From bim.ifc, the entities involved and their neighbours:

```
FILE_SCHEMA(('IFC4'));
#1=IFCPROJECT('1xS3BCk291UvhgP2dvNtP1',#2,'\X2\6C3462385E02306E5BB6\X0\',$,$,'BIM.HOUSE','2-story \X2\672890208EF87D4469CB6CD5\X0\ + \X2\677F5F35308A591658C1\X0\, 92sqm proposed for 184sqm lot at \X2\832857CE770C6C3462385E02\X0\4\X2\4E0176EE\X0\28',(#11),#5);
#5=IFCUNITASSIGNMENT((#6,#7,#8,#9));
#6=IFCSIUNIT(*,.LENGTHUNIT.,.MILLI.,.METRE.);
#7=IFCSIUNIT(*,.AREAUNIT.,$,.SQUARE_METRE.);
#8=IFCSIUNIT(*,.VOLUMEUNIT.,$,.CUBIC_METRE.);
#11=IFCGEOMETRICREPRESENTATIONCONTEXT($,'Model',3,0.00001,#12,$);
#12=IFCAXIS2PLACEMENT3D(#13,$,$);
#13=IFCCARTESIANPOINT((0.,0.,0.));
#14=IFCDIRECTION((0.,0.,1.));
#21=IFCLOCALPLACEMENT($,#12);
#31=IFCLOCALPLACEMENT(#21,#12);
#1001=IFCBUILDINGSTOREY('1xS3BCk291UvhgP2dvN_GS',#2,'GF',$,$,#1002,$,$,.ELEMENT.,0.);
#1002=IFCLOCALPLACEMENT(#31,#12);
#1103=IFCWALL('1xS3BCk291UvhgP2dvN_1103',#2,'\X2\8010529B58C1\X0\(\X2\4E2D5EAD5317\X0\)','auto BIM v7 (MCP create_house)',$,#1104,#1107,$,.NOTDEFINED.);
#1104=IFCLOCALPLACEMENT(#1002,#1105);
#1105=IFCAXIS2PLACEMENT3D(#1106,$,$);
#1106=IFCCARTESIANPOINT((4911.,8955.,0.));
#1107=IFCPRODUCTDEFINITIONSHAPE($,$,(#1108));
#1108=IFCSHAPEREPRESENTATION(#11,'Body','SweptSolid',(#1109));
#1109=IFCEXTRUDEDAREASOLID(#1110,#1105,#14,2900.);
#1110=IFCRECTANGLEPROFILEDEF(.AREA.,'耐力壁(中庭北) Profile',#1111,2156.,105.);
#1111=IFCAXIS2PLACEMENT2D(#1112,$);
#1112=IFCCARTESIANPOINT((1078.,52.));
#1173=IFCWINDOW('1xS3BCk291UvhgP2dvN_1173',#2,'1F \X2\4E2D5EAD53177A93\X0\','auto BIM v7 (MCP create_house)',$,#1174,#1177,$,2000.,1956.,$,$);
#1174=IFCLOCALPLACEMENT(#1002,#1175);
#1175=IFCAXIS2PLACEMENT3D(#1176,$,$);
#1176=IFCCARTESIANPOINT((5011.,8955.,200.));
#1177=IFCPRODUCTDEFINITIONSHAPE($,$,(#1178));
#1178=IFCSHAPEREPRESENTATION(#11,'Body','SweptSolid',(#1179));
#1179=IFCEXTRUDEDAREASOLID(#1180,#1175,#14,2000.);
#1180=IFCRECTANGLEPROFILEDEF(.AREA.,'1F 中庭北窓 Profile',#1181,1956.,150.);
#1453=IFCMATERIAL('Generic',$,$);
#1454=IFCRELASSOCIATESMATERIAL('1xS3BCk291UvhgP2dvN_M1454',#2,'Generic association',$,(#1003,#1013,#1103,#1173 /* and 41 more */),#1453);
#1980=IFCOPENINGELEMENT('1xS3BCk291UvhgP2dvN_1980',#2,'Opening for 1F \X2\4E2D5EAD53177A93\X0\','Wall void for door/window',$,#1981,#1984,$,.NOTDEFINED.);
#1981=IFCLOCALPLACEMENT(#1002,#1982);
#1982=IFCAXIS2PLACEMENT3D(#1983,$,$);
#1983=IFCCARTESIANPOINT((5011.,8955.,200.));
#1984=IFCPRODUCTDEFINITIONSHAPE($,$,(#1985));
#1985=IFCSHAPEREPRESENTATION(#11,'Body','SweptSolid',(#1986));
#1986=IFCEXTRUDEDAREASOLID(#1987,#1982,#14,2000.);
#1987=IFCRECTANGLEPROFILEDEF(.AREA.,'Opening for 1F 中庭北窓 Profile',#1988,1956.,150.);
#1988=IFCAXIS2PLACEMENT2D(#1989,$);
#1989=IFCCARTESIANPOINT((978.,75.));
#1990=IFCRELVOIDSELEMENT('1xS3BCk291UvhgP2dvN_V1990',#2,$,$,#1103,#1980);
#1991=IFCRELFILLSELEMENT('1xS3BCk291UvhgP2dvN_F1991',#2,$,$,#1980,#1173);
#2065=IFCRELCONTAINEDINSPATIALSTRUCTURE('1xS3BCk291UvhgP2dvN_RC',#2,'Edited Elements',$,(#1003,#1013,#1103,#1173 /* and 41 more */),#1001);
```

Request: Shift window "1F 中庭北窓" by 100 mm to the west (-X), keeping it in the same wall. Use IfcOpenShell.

```python
import ifcopenshell
import ifcopenshell.api.geometry
import ifcopenshell.util.placement
import ifcopenshell.util.unit

model = ifcopenshell.open("bim.ifc")
unit_scale = ifcopenshell.util.unit.calculate_unit_scale(model)

window = model.by_guid("1xS3BCk291UvhgP2dvN_1173")
opening = window.FillsVoids[0].RelatingOpeningElement
wall = opening.VoidsElements[0].RelatingBuildingElement

wall_matrix = ifcopenshell.util.placement.get_local_placement(wall.ObjectPlacement)
shift = wall_matrix[:3, 0] * -0.1 / unit_scale
before = ifcopenshell.util.placement.get_local_placement(window.ObjectPlacement)[:3, 3].copy()

# The window is not placed relative to its opening, so move both.
for product in (opening, window):
    matrix = ifcopenshell.util.placement.get_local_placement(product.ObjectPlacement)
    matrix[:3, 3] += shift
    ifcopenshell.api.geometry.edit_object_placement(model, product=product, matrix=matrix, is_si=False)

after = ifcopenshell.util.placement.get_local_placement(window.ObjectPlacement)[:3, 3]
print("window moved by", (after - before).round(3) + 0.0)

model.write("bim_edited.ifc")
```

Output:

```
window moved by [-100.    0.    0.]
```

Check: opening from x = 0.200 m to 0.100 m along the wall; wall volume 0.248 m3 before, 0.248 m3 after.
